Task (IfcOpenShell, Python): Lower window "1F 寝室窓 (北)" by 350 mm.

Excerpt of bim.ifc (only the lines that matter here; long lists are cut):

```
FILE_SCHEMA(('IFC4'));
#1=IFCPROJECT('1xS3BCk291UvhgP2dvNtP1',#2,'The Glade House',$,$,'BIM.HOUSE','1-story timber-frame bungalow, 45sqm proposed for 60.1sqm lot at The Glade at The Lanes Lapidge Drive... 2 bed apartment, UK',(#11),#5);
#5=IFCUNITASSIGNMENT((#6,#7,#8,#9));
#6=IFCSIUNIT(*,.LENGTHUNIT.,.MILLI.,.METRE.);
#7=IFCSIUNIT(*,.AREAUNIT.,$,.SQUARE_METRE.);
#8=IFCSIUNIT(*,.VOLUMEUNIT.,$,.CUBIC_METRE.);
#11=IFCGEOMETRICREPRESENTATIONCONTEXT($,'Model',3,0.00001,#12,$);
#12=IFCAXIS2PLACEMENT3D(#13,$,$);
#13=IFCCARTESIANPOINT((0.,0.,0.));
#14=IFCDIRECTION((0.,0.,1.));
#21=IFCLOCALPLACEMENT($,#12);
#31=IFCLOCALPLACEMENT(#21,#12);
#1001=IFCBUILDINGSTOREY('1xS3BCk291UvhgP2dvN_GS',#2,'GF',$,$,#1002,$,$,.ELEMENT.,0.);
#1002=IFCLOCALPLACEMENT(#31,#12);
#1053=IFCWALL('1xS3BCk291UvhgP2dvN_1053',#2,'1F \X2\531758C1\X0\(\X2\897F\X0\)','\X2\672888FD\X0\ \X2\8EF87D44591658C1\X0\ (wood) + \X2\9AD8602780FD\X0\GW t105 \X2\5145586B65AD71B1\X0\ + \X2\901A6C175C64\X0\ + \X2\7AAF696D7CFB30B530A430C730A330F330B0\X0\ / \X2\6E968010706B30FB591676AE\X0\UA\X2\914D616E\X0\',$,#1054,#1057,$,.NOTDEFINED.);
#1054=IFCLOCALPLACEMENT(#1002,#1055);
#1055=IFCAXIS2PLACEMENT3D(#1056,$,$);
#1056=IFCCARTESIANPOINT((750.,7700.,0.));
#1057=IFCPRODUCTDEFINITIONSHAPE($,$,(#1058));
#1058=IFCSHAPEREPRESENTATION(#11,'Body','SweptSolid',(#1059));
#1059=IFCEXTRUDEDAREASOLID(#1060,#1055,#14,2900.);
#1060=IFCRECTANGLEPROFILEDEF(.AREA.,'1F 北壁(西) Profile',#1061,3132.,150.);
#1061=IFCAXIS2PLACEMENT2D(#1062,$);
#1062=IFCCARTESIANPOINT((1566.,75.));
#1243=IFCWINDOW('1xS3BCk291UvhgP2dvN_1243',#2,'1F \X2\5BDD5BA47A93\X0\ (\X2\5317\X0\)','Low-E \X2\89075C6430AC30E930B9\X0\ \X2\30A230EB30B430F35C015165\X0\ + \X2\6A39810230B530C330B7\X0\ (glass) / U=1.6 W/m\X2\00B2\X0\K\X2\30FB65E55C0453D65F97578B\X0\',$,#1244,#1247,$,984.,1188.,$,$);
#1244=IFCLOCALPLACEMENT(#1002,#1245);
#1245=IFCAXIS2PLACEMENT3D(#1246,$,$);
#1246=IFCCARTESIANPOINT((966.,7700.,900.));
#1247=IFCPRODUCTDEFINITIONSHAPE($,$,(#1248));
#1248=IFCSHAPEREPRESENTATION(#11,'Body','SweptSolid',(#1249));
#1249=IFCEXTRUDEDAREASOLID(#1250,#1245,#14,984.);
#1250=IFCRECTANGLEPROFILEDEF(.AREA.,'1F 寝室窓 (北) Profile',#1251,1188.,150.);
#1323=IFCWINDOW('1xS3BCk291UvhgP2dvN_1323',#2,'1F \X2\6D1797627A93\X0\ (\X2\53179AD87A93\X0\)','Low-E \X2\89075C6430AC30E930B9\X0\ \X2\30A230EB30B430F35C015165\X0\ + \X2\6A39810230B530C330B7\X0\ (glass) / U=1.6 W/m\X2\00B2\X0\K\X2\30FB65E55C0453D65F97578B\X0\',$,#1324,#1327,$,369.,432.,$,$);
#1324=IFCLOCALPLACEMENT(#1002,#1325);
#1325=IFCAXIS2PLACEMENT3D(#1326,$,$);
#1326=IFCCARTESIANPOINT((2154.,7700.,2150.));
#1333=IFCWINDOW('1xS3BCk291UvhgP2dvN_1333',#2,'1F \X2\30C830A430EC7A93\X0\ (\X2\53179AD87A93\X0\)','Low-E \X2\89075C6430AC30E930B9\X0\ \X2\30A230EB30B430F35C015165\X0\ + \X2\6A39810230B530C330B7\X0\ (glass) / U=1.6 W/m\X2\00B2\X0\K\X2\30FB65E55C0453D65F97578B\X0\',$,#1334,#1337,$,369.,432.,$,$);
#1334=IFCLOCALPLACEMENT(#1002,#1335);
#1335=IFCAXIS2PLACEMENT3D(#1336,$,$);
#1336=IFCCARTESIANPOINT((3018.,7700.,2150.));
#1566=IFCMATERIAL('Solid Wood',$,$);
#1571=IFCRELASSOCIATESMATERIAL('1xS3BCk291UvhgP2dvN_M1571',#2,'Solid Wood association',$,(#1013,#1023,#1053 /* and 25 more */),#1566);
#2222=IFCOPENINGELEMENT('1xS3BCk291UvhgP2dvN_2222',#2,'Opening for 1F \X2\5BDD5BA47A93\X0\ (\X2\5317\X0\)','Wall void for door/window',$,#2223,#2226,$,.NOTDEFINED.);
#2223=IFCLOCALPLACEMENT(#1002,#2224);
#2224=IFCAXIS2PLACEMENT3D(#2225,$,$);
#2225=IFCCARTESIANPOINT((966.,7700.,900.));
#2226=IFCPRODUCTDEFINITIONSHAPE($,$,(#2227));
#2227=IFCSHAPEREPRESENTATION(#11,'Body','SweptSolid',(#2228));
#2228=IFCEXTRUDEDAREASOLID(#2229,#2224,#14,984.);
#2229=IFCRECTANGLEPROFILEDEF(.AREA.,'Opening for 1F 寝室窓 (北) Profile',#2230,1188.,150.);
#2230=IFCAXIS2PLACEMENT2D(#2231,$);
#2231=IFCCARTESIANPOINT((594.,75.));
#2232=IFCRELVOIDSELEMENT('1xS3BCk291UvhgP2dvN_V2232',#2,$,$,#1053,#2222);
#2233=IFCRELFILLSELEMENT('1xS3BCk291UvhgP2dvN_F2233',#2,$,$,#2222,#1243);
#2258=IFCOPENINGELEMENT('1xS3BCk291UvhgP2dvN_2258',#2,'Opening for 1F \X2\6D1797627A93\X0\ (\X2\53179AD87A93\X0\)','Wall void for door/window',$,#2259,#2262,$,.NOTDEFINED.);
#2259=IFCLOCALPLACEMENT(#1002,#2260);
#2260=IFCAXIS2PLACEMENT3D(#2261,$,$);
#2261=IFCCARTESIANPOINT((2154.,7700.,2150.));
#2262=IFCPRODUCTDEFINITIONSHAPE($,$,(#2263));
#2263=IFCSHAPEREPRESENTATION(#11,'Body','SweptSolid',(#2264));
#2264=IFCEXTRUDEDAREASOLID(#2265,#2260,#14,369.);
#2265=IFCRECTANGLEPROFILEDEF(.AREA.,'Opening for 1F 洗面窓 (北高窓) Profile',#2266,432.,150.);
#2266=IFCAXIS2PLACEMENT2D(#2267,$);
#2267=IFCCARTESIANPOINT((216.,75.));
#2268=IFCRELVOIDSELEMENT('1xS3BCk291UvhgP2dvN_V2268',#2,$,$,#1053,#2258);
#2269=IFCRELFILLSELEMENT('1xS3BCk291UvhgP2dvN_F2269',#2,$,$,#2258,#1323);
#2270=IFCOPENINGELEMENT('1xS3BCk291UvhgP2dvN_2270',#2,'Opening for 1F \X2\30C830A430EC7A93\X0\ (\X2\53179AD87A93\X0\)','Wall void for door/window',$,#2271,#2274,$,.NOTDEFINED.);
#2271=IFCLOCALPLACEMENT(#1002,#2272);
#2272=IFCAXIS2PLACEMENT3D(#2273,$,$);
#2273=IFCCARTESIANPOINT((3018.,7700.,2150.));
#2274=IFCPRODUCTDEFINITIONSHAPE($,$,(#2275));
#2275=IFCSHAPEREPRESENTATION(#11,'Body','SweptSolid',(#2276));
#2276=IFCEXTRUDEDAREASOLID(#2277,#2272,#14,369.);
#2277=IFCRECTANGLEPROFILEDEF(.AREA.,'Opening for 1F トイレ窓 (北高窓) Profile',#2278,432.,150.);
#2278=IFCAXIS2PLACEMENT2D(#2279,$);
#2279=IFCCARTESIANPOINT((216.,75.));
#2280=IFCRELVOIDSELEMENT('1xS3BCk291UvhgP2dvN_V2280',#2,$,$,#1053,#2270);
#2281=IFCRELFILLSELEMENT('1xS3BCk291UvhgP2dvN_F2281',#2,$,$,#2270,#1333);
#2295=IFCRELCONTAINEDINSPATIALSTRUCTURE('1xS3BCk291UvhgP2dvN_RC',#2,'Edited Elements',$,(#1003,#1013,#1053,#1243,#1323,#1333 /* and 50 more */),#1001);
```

```python
import numpy as np
import ifcopenshell
import ifcopenshell.api.geometry
import ifcopenshell.util.placement
import ifcopenshell.util.unit

model = ifcopenshell.open("bim.ifc")
unit_scale = ifcopenshell.util.unit.calculate_unit_scale(model)

window = model.by_id(1243)
opening = window.FillsVoids[0].RelatingOpeningElement
dz = -0.35 / unit_scale

shift = np.array([0.0, 0.0, dz])
# The window is not placed relative to its opening, so move both.
for product in (opening, window):
    matrix = ifcopenshell.util.placement.get_local_placement(product.ObjectPlacement)
    matrix[:3, 3] += shift
    ifcopenshell.api.geometry.edit_object_placement(model, product=product, matrix=matrix, is_si=False)

print(f"moved by {dz * unit_scale:+.3f} m")

model.write("bim_rev.ifc")
```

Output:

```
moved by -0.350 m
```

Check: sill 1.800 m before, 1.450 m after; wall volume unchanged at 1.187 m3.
